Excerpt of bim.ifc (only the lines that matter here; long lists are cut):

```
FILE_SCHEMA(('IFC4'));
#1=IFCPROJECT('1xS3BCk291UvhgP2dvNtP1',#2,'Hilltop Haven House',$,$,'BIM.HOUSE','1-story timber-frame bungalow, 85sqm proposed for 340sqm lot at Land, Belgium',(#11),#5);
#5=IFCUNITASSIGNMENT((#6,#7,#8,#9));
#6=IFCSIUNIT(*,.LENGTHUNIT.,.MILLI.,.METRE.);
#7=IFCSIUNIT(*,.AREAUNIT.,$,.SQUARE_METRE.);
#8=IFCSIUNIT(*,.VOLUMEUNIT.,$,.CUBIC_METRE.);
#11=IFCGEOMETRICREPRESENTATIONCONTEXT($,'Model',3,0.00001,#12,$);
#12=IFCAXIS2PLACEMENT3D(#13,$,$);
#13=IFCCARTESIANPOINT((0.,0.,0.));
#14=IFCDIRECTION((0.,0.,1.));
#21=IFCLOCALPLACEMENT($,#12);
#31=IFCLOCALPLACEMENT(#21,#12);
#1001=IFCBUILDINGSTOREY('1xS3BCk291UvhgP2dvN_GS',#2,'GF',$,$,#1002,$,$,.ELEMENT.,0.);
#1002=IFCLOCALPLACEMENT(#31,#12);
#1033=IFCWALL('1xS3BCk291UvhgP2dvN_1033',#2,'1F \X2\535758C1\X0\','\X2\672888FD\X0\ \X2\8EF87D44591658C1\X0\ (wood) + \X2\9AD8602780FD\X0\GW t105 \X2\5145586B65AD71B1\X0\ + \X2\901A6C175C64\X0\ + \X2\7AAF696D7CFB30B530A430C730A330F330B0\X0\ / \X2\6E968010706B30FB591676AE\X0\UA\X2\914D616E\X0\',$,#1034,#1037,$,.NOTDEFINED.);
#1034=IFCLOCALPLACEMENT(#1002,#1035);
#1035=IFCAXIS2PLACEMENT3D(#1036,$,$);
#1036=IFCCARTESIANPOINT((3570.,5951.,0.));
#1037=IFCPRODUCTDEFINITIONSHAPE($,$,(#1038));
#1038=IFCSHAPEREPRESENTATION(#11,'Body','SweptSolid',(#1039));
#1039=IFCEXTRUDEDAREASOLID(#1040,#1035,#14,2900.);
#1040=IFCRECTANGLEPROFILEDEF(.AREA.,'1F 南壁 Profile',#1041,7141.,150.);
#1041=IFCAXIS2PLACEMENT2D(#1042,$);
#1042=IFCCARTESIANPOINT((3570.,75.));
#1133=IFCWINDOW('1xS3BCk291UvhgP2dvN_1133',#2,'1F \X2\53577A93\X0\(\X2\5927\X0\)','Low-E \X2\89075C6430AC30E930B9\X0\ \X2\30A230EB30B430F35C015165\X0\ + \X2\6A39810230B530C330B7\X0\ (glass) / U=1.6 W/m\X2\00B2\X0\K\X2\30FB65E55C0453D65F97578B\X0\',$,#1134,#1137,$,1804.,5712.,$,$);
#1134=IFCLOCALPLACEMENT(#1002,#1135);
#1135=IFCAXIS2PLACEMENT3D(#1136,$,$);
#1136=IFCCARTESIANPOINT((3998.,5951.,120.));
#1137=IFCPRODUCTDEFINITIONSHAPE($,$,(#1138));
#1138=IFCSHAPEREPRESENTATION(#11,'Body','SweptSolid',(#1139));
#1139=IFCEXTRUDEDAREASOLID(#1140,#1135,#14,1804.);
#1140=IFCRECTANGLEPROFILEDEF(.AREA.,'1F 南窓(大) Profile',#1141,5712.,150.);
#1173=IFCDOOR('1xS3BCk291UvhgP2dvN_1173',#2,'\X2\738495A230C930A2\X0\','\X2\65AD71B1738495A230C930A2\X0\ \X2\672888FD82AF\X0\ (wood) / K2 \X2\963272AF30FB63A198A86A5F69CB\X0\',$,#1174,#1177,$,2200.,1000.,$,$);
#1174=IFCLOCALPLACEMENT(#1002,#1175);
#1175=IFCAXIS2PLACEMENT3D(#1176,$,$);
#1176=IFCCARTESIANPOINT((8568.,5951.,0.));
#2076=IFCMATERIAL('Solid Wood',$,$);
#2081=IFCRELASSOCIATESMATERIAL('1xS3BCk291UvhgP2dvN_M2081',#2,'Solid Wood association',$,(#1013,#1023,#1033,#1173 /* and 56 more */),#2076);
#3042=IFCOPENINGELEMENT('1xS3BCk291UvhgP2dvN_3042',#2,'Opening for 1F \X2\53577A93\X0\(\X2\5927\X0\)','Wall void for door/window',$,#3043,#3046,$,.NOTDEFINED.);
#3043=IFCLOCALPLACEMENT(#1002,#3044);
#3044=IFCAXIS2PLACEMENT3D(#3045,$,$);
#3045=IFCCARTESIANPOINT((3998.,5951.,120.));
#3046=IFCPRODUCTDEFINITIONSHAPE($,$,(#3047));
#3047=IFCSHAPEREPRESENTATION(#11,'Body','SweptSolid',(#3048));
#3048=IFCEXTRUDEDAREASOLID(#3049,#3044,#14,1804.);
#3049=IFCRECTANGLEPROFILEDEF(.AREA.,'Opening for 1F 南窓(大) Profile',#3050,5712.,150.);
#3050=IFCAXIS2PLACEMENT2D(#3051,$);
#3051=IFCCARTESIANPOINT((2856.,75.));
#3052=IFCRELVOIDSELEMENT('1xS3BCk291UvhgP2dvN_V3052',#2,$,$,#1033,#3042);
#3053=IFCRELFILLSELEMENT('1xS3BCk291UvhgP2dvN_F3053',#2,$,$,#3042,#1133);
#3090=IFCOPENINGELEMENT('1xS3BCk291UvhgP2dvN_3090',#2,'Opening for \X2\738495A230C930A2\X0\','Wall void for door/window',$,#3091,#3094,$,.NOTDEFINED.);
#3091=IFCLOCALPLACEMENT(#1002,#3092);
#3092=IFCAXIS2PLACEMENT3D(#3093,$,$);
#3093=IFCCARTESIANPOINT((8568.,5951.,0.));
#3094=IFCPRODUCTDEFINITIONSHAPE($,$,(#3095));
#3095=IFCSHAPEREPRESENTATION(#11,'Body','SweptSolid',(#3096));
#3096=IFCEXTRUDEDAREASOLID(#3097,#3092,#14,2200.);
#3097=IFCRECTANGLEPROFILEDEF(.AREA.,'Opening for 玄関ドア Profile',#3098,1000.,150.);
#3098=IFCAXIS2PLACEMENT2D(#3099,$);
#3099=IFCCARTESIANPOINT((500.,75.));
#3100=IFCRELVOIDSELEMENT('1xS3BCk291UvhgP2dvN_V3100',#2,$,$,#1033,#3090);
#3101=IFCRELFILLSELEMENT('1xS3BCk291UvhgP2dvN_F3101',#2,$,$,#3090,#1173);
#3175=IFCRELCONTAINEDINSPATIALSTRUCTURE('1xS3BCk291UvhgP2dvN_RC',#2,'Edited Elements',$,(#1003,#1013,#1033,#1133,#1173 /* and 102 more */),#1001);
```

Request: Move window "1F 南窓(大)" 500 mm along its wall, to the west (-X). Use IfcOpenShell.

```python
import ifcopenshell
import ifcopenshell.api.geometry
import ifcopenshell.util.placement
import ifcopenshell.util.unit

model = ifcopenshell.open("bim.ifc")
unit_scale = ifcopenshell.util.unit.calculate_unit_scale(model)

window = model.by_guid("1xS3BCk291UvhgP2dvN_1133")
opening = window.FillsVoids[0].RelatingOpeningElement
wall = opening.VoidsElements[0].RelatingBuildingElement

wall_matrix = ifcopenshell.util.placement.get_local_placement(wall.ObjectPlacement)
shift = wall_matrix[:3, 0] * -0.5 / unit_scale
before = ifcopenshell.util.placement.get_local_placement(window.ObjectPlacement)[:3, 3].copy()

# The window is not placed relative to its opening, so move both.
for product in (opening, window):
    matrix = ifcopenshell.util.placement.get_local_placement(product.ObjectPlacement)
    matrix[:3, 3] += shift
    ifcopenshell.api.geometry.edit_object_placement(model, product=product, matrix=matrix, is_si=False)

after = ifcopenshell.util.placement.get_local_placement(window.ObjectPlacement)[:3, 3]
print("window moved by", (after - before).round(3) + 0.0)

model.write("bim_rev.ifc")
```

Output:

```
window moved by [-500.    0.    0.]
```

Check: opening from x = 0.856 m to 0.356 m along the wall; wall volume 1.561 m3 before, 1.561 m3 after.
